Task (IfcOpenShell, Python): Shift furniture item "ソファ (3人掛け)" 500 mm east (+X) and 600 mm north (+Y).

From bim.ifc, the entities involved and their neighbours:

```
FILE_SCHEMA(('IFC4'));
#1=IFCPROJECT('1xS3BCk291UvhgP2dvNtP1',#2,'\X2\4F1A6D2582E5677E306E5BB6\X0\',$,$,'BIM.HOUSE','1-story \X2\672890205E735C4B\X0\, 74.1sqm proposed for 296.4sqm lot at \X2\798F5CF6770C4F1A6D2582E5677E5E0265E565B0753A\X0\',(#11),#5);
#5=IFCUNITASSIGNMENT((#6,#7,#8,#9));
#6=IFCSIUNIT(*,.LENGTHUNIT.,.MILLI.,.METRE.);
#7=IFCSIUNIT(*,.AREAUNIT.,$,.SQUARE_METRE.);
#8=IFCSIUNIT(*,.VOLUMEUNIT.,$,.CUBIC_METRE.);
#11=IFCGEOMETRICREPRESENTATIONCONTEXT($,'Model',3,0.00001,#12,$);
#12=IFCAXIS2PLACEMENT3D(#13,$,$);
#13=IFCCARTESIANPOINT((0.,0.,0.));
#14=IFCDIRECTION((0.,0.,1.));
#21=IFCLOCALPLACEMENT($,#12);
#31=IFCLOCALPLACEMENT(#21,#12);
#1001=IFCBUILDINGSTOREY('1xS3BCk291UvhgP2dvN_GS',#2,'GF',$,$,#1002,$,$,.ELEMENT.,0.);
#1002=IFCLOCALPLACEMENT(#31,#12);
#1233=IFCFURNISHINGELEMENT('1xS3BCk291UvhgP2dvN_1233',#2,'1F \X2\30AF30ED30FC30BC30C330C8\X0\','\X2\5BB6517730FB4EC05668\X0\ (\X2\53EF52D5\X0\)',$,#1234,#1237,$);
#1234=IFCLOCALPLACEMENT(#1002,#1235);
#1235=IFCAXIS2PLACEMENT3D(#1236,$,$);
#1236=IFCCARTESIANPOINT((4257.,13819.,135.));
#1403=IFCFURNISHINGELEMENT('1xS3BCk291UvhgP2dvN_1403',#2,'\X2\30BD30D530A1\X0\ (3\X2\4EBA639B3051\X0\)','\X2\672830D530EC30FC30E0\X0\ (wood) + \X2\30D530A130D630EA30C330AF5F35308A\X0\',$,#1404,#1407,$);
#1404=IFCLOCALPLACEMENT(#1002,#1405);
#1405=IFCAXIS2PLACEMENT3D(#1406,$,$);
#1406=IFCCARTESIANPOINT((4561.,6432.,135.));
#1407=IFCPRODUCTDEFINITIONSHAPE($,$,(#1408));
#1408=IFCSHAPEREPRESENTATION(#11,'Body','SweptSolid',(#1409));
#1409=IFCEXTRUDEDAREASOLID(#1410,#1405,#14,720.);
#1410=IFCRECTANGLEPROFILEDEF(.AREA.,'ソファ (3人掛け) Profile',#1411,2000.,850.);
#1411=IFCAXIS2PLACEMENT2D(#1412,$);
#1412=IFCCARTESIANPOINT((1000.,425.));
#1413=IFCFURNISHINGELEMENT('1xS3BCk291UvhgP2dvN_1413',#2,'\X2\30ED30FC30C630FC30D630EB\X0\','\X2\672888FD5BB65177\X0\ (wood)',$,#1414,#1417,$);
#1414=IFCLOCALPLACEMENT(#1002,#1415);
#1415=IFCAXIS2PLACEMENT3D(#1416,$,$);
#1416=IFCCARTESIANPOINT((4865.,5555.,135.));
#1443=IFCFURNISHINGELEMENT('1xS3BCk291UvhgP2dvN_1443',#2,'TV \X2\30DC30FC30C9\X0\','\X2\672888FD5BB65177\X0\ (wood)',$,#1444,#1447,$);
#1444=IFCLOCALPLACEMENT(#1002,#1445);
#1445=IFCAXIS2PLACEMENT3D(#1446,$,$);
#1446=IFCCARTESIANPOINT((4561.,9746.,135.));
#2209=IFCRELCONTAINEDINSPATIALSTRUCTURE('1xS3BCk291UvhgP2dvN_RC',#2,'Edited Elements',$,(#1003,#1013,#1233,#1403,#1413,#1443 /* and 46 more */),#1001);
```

```python
import ifcopenshell
import ifcopenshell.api.geometry
import ifcopenshell.util.placement

model = ifcopenshell.open("bim.ifc")

item = model.by_id(1403)
matrix = ifcopenshell.util.placement.get_local_placement(item.ObjectPlacement)
matrix[0, 3] += 500.0
matrix[1, 3] += 600.0
ifcopenshell.api.geometry.edit_object_placement(model, product=item, matrix=matrix, is_si=False)

print(ifcopenshell.util.placement.get_local_placement(item.ObjectPlacement).round(3) + 0.0)

model.write("bim_v2.ifc")
```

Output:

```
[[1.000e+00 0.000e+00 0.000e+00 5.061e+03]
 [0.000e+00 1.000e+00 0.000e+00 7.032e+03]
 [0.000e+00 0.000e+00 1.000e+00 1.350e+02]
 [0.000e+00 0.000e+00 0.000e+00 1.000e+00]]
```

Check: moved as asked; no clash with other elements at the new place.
